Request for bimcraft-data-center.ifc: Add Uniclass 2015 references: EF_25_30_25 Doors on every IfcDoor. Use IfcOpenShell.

First a look at what the model holds.

```python
import ifcopenshell

model = ifcopenshell.open("bimcraft-data-center.ifc")
print(model.schema)
print("classifications:", [c.Name for c in model.by_type("IfcClassification")])
for ifc_class in ("IfcDoor", "IfcRoof", "IfcStair", "IfcWall", "IfcWindow"):
    print(ifc_class, len(model.by_type(ifc_class)))
```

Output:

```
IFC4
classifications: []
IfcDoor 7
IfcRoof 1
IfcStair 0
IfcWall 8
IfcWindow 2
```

```python
import ifcopenshell
import ifcopenshell.api.classification

model = ifcopenshell.open("bimcraft-data-center.ifc")

system = ifcopenshell.api.classification.add_classification(model, classification="Uniclass 2015")

codes = {
    "IfcDoor": ("EF_25_30_25", "Doors"),
}
for ifc_class, (code, name) in codes.items():
    products = model.by_type(ifc_class)
    ifcopenshell.api.classification.add_reference(
        model, products=products, classification=system, identification=code, name=name
    )
    print(code, len(products))

model.write("bimcraft-data-center_v2.ifc")
```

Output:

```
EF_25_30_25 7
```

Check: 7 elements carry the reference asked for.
